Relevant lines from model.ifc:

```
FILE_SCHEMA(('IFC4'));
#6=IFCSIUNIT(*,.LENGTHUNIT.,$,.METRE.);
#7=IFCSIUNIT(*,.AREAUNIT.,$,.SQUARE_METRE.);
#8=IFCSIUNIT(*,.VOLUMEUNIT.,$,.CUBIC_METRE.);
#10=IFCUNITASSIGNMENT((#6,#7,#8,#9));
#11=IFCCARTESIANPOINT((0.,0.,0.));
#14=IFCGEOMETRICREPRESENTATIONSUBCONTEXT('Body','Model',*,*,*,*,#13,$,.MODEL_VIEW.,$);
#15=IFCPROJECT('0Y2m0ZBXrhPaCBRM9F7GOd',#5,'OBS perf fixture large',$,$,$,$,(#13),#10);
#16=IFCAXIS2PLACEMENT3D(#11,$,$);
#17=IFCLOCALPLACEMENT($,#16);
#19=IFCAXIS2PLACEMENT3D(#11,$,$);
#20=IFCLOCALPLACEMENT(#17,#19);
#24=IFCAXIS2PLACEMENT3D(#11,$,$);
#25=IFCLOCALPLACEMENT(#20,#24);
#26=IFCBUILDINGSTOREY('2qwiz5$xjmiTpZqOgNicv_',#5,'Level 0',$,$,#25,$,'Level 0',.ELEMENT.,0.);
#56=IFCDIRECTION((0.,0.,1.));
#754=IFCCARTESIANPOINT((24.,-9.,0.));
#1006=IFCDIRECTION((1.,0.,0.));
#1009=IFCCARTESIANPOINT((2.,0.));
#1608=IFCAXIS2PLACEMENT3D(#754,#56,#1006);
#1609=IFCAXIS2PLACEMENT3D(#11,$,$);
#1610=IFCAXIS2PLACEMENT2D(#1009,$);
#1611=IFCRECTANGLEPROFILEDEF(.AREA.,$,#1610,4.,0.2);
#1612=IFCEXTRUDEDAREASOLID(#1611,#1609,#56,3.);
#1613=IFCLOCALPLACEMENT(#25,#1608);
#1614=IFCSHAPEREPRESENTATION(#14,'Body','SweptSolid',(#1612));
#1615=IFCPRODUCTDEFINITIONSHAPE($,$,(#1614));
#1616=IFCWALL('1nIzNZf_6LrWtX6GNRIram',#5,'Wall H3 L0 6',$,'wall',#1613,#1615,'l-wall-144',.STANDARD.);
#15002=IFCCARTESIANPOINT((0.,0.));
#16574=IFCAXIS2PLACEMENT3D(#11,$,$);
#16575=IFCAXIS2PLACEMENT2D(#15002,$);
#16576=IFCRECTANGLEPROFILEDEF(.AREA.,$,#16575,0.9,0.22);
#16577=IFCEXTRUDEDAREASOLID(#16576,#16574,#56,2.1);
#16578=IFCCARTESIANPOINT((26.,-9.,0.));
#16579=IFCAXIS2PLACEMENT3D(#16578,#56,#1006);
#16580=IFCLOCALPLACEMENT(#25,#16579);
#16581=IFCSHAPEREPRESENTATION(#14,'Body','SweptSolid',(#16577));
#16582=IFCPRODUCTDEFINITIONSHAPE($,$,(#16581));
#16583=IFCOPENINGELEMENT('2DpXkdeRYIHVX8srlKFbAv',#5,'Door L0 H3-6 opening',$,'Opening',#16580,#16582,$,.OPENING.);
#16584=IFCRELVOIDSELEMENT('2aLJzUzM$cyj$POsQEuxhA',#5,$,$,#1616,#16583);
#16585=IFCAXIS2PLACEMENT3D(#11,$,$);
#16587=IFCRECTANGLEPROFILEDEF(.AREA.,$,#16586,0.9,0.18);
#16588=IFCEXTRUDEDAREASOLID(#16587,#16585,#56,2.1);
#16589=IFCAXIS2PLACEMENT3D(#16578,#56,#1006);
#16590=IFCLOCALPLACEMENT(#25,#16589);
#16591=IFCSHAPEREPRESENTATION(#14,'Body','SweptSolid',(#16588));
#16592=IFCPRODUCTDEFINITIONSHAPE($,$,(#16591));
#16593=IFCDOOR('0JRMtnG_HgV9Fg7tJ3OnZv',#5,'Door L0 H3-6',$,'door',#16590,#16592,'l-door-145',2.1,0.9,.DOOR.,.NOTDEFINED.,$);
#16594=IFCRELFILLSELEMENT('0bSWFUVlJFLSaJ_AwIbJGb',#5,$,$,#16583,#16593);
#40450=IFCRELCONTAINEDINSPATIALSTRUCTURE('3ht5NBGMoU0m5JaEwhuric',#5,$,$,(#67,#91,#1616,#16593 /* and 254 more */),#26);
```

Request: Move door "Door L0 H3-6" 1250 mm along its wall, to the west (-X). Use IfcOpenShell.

```python
import ifcopenshell
import ifcopenshell.api.geometry
import ifcopenshell.util.placement
import ifcopenshell.util.unit

model = ifcopenshell.open("model.ifc")
unit_scale = ifcopenshell.util.unit.calculate_unit_scale(model)

door = model.by_id(16593)
opening = door.FillsVoids[0].RelatingOpeningElement
wall = opening.VoidsElements[0].RelatingBuildingElement

wall_matrix = ifcopenshell.util.placement.get_local_placement(wall.ObjectPlacement)
shift = wall_matrix[:3, 0] * -1.25 / unit_scale
before = ifcopenshell.util.placement.get_local_placement(door.ObjectPlacement)[:3, 3].copy()

# The door is not placed relative to its opening, so move both.
for product in (opening, door):
    matrix = ifcopenshell.util.placement.get_local_placement(product.ObjectPlacement)
    matrix[:3, 3] += shift
    ifcopenshell.api.geometry.edit_object_placement(model, product=product, matrix=matrix, is_si=False)

after = ifcopenshell.util.placement.get_local_placement(door.ObjectPlacement)[:3, 3]
print("door moved by", (after - before).round(3) + 0.0)

model.write("model_updated.ifc")
```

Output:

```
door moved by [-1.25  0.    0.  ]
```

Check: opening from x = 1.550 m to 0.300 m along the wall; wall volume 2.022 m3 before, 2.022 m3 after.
